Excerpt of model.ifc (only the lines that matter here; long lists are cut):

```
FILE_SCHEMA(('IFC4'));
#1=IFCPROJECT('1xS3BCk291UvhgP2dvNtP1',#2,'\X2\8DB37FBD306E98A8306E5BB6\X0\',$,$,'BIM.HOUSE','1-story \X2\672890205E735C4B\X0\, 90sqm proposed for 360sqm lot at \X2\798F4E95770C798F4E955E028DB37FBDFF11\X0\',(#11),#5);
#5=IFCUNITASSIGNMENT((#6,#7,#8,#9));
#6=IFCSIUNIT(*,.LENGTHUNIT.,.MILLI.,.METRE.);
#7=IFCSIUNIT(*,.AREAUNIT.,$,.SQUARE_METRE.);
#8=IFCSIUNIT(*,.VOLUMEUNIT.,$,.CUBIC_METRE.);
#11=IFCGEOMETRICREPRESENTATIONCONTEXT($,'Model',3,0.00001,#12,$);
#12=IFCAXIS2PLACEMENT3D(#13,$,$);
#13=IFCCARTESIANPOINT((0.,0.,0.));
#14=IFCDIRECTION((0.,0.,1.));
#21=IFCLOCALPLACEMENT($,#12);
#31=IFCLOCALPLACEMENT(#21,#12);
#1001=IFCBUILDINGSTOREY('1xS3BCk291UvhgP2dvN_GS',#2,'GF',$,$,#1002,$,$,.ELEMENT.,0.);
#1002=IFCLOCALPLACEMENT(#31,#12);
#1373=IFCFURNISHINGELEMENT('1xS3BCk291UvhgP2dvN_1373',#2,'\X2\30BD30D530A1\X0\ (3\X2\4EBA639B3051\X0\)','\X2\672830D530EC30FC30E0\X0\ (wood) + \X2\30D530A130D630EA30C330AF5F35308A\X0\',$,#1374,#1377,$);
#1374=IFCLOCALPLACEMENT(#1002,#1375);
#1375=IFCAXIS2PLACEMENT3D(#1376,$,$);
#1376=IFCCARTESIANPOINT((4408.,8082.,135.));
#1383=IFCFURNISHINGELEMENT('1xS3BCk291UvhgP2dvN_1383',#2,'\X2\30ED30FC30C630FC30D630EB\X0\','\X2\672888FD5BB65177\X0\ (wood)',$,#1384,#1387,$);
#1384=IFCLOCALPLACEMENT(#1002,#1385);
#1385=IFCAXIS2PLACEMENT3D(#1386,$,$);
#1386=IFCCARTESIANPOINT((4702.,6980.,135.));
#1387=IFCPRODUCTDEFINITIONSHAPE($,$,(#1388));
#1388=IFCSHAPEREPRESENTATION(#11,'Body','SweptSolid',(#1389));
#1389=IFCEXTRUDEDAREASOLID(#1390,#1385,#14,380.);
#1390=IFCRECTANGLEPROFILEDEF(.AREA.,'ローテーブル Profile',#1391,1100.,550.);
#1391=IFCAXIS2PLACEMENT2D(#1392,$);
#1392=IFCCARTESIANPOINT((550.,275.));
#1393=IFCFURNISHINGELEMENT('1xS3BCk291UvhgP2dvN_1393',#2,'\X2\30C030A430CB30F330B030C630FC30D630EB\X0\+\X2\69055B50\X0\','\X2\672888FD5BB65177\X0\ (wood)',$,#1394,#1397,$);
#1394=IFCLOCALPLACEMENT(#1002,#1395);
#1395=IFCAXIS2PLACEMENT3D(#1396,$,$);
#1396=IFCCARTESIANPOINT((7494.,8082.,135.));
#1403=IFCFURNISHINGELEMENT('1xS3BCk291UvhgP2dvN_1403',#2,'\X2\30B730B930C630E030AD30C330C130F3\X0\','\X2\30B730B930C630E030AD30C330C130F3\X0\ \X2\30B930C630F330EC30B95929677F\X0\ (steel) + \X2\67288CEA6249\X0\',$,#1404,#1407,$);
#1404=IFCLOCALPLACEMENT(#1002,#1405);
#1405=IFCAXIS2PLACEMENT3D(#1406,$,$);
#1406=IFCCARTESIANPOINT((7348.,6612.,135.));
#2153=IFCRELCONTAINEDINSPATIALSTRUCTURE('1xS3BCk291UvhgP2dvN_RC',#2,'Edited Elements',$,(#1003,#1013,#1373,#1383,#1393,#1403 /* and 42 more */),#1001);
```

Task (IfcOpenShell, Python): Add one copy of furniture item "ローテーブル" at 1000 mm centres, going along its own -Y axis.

```python
import ifcopenshell
import ifcopenshell.api.geometry
import ifcopenshell.api.root
import ifcopenshell.util.element
import ifcopenshell.util.placement
import ifcopenshell.util.unit

model = ifcopenshell.open("model.ifc")
unit_scale = ifcopenshell.util.unit.calculate_unit_scale(model)


def reuse_history(source, copy):
    """copy_class also copies each property set's owner history, people and application; keep the originals."""
    for rel in copy.IsDefinedBy:
        if rel.is_a("IfcRelDefinesByProperties") and (history := rel.RelatingPropertyDefinition.OwnerHistory):
            rel.RelatingPropertyDefinition.OwnerHistory = source.OwnerHistory
            ifcopenshell.util.element.remove_deep2(model, history)


source = model.by_guid("1xS3BCk291UvhgP2dvN_1383")
base = ifcopenshell.util.placement.get_local_placement(source.ObjectPlacement)
step = -base[:3, 1] * 1 / unit_scale

for i in range(1, 2):
    copy = ifcopenshell.api.root.copy_class(model, product=source)
    copy.Representation = ifcopenshell.util.element.copy_deep(
        model, source.Representation, exclude=["IfcGeometricRepresentationContext", "IfcRepresentationMap"]
    )
    reuse_history(source, copy)
    matrix = base.copy()
    matrix[:3, 3] += i * step
    print("added at", matrix[:3, 3].round(3) + 0.0)
    ifcopenshell.api.geometry.edit_object_placement(model, product=copy, matrix=matrix, is_si=False)

model.write("model_updated.ifc")
```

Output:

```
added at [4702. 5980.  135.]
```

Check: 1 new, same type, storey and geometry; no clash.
